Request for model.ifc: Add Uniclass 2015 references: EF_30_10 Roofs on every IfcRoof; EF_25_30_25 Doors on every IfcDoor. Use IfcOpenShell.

First a look at what the model holds.

```python
import ifcopenshell

model = ifcopenshell.open("model.ifc")
print(model.schema)
print("classifications:", [c.Name for c in model.by_type("IfcClassification")])
for ifc_class in ("IfcDoor", "IfcRoof", "IfcStair", "IfcWall", "IfcWindow"):
    print(ifc_class, len(model.by_type(ifc_class)))
```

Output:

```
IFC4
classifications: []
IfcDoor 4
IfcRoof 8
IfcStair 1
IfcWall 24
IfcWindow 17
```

```python
import ifcopenshell
import ifcopenshell.api.classification

model = ifcopenshell.open("model.ifc")

system = ifcopenshell.api.classification.add_classification(model, classification="Uniclass 2015")

codes = {
    "IfcRoof": ("EF_30_10", "Roofs"),
    "IfcDoor": ("EF_25_30_25", "Doors"),
}
for ifc_class, (code, name) in codes.items():
    products = model.by_type(ifc_class)
    ifcopenshell.api.classification.add_reference(
        model, products=products, classification=system, identification=code, name=name
    )
    print(code, len(products))

model.write("model_v2.ifc")
```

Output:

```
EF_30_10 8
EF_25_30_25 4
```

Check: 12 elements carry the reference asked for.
